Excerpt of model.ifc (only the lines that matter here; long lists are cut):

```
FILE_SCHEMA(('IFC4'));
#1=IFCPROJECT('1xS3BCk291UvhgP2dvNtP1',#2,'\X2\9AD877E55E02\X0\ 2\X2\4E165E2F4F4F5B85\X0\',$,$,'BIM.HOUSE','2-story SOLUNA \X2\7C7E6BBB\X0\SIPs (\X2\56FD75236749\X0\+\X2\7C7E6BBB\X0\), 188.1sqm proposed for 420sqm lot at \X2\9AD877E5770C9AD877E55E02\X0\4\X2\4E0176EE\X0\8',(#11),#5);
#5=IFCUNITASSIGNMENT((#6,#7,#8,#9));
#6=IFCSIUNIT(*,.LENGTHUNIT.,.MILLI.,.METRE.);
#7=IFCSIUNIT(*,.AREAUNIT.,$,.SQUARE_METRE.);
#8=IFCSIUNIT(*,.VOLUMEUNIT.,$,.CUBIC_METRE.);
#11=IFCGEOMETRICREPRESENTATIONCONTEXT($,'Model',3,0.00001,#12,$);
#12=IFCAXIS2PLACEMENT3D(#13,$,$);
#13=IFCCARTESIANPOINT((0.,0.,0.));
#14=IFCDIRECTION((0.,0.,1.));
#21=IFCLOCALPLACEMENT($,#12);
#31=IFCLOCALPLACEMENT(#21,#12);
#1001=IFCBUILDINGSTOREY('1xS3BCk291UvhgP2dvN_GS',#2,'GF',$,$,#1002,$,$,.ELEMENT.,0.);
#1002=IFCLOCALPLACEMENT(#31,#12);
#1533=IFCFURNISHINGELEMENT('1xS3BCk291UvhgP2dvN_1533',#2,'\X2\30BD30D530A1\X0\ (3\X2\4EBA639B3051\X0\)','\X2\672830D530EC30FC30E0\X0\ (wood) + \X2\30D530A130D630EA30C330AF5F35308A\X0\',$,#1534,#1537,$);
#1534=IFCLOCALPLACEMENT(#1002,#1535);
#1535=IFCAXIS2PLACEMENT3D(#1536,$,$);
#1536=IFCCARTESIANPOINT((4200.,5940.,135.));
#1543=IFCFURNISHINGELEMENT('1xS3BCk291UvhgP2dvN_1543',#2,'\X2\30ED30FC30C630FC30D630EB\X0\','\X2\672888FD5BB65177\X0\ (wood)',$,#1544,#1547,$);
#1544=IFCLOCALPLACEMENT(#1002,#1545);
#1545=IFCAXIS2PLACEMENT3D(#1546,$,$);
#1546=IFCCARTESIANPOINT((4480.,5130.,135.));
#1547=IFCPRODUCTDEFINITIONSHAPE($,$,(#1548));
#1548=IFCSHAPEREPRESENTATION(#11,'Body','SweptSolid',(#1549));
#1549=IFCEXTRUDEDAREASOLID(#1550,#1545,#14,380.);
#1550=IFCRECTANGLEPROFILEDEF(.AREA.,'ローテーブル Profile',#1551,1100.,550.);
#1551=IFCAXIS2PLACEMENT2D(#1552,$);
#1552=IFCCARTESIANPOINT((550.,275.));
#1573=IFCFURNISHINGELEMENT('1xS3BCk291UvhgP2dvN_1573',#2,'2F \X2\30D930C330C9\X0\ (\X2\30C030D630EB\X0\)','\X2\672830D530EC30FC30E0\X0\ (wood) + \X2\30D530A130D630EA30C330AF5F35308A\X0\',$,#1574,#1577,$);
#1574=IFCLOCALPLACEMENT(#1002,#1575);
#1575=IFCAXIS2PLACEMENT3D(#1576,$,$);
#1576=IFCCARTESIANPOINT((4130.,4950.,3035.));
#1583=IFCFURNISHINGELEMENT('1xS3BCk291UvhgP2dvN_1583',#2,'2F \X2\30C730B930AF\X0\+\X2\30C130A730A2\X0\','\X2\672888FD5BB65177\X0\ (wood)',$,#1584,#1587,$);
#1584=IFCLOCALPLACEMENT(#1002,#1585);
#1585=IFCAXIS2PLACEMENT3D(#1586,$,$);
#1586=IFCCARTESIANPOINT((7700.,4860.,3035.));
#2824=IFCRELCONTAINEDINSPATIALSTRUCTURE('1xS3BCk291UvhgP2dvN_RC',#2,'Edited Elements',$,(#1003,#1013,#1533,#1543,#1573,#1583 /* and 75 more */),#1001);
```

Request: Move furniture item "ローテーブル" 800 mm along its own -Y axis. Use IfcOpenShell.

```python
import ifcopenshell
import ifcopenshell.api.geometry
import ifcopenshell.util.placement
import ifcopenshell.util.unit

model = ifcopenshell.open("model.ifc")
unit_scale = ifcopenshell.util.unit.calculate_unit_scale(model)

item = model.by_guid("1xS3BCk291UvhgP2dvN_1543")
matrix = ifcopenshell.util.placement.get_local_placement(item.ObjectPlacement)
matrix[:3, 3] -= matrix[:3, 1] * 0.8 / unit_scale
ifcopenshell.api.geometry.edit_object_placement(model, product=item, matrix=matrix, is_si=False)

print(ifcopenshell.util.placement.get_local_placement(item.ObjectPlacement).round(3) + 0.0)

model.write("model_v2.ifc")
```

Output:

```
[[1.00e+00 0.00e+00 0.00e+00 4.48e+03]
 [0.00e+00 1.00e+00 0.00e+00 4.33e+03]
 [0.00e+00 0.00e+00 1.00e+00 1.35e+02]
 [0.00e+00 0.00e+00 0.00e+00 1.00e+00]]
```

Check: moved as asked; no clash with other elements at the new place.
